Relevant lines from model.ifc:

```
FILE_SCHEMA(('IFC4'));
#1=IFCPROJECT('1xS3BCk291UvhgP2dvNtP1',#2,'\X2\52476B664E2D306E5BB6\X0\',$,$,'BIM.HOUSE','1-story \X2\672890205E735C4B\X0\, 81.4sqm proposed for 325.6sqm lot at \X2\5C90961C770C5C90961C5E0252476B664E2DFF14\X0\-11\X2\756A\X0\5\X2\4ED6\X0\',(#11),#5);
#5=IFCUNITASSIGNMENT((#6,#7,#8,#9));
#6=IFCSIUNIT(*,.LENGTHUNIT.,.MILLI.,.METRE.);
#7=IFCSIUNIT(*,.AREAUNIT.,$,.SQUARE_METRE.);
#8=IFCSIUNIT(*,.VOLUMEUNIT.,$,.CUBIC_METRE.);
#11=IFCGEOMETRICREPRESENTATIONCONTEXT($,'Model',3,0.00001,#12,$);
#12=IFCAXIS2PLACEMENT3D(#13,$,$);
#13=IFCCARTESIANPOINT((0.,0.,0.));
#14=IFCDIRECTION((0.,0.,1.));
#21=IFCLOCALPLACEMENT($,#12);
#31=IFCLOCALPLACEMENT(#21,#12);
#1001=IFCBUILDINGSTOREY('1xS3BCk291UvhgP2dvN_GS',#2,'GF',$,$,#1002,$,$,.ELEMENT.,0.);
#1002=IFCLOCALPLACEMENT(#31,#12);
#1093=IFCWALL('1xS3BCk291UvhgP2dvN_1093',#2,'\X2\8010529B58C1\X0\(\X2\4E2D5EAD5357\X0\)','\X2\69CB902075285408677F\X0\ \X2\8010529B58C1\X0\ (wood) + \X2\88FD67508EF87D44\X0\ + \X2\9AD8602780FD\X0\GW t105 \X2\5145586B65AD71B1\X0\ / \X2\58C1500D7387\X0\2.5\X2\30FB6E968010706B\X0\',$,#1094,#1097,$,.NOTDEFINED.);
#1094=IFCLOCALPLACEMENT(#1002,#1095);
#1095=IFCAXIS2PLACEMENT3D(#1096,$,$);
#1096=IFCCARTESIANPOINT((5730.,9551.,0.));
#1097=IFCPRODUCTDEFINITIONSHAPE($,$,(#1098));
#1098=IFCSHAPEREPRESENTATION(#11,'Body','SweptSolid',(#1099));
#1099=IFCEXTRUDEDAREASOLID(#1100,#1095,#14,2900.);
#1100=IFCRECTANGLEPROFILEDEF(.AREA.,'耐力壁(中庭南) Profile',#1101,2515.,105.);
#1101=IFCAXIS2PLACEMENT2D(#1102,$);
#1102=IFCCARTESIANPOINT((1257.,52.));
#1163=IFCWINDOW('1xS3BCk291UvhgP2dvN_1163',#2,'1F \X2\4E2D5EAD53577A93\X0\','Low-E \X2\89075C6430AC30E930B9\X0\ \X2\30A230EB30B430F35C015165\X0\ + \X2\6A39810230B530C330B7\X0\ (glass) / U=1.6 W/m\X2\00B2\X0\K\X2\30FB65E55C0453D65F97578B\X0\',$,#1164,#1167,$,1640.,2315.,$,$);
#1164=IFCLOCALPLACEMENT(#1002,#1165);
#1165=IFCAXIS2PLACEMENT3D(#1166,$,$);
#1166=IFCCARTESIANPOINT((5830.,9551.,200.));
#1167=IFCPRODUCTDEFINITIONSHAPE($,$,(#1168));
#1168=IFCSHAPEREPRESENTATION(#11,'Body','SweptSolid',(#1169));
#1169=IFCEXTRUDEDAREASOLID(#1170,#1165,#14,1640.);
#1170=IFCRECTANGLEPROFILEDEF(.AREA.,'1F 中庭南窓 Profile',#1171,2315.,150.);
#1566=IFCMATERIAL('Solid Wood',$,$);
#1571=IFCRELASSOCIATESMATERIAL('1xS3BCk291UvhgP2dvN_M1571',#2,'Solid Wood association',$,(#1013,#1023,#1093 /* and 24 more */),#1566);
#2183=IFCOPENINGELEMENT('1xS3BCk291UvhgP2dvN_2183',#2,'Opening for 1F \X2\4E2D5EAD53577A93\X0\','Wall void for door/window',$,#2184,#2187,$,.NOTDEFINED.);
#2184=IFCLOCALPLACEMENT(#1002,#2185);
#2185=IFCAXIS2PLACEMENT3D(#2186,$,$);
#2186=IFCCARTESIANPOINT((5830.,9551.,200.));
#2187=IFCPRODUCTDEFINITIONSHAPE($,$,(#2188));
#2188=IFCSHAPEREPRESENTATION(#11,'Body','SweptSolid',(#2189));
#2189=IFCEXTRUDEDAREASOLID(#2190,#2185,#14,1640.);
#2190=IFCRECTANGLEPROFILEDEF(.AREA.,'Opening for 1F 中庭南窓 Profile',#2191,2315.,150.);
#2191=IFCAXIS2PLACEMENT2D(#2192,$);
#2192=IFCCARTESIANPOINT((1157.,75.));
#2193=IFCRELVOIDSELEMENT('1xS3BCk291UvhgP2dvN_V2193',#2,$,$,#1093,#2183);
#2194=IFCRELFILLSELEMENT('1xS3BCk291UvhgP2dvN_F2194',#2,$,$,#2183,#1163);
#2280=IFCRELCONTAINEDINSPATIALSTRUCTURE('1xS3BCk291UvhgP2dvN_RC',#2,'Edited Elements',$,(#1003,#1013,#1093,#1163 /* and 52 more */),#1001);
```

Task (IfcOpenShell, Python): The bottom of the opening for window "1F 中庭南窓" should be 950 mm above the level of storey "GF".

```python
import numpy as np
import ifcopenshell
import ifcopenshell.api.geometry
import ifcopenshell.geom
import ifcopenshell.util.element
import ifcopenshell.util.placement
import ifcopenshell.util.shape
import ifcopenshell.util.unit

model = ifcopenshell.open("model.ifc")
unit_scale = ifcopenshell.util.unit.calculate_unit_scale(model)

window = model.by_id(1163)
opening = window.FillsVoids[0].RelatingOpeningElement
storey = ifcopenshell.util.element.get_container(window, ifc_class="IfcBuildingStorey")
level = ifcopenshell.util.placement.get_local_placement(storey.ObjectPlacement)[2, 3]

# The opening's origin need not be at the sill, so measure its lowest point.
shape = ifcopenshell.geom.create_shape(ifcopenshell.geom.settings(), opening)
bottom = ifcopenshell.util.shape.get_shape_bottom_elevation(shape, shape.geometry) / unit_scale
dz = level + 0.95 / unit_scale - bottom

shift = np.array([0.0, 0.0, dz])
# The window is not placed relative to its opening, so move both.
for product in (opening, window):
    matrix = ifcopenshell.util.placement.get_local_placement(product.ObjectPlacement)
    matrix[:3, 3] += shift
    ifcopenshell.api.geometry.edit_object_placement(model, product=product, matrix=matrix, is_si=False)

print(f"moved by {dz * unit_scale:+.3f} m")

model.write("model-out.ifc")
```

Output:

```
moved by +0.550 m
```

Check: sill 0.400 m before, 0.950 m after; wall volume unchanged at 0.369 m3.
